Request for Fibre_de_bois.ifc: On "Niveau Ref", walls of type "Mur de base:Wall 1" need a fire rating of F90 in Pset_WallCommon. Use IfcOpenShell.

First a look at what the model holds.

```python
import ifcopenshell
import ifcopenshell.util.element

model = ifcopenshell.open("Fibre_de_bois.ifc")
print(model.schema)
storey = next(s for s in model.by_type("IfcBuildingStorey") if s.Name == "Niveau Ref")
walls = [e for e in ifcopenshell.util.element.get_decomposition(storey) if e.is_a("IfcWall")]
seen = {}
for e in walls:
    element_type = ifcopenshell.util.element.get_type(e)
    key = (element_type.Name if element_type != e and element_type else None, ifcopenshell.util.element.get_pset(e, "Pset_WallCommon", "FireRating"))
    seen[key] = seen.get(key, 0) + 1
for (name, value), count in sorted(seen.items(), key=str):
    print(count, "x", name, "|", value)
```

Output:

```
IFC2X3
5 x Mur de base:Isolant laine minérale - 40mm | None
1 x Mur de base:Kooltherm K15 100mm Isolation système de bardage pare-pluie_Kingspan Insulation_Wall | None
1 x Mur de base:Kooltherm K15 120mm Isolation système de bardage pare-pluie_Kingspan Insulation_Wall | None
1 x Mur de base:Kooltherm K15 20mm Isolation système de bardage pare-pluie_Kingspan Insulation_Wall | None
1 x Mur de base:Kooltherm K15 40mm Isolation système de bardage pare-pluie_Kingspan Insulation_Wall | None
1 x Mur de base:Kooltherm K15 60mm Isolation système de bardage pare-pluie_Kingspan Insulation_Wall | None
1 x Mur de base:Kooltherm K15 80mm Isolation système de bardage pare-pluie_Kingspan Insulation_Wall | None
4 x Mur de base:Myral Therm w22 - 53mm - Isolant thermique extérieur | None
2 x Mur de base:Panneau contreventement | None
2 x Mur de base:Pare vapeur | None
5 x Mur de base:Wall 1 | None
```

```python
import ifcopenshell
import ifcopenshell.api.pset
import ifcopenshell.util.element

model = ifcopenshell.open("Fibre_de_bois.ifc")

storey = next(s for s in model.by_type("IfcBuildingStorey") if s.Name == "Niveau Ref")
walls = [e for e in ifcopenshell.util.element.get_decomposition(storey) if e.is_a("IfcWall")]

count = 0
for e in walls:
    element_type = ifcopenshell.util.element.get_type(e)
    if element_type in (None, e) or element_type.Name != "Mur de base:Wall 1":
        continue
    # add_pset returns the element's existing set when there is one.
    pset = ifcopenshell.api.pset.add_pset(model, product=e, name="Pset_WallCommon")
    ifcopenshell.api.pset.edit_pset(model, pset=pset, properties={"FireRating": "F90"})
    count += 1

print(count, "walls updated")

model.write("Fibre_de_bois_v2.ifc")
```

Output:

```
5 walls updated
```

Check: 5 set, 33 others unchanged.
